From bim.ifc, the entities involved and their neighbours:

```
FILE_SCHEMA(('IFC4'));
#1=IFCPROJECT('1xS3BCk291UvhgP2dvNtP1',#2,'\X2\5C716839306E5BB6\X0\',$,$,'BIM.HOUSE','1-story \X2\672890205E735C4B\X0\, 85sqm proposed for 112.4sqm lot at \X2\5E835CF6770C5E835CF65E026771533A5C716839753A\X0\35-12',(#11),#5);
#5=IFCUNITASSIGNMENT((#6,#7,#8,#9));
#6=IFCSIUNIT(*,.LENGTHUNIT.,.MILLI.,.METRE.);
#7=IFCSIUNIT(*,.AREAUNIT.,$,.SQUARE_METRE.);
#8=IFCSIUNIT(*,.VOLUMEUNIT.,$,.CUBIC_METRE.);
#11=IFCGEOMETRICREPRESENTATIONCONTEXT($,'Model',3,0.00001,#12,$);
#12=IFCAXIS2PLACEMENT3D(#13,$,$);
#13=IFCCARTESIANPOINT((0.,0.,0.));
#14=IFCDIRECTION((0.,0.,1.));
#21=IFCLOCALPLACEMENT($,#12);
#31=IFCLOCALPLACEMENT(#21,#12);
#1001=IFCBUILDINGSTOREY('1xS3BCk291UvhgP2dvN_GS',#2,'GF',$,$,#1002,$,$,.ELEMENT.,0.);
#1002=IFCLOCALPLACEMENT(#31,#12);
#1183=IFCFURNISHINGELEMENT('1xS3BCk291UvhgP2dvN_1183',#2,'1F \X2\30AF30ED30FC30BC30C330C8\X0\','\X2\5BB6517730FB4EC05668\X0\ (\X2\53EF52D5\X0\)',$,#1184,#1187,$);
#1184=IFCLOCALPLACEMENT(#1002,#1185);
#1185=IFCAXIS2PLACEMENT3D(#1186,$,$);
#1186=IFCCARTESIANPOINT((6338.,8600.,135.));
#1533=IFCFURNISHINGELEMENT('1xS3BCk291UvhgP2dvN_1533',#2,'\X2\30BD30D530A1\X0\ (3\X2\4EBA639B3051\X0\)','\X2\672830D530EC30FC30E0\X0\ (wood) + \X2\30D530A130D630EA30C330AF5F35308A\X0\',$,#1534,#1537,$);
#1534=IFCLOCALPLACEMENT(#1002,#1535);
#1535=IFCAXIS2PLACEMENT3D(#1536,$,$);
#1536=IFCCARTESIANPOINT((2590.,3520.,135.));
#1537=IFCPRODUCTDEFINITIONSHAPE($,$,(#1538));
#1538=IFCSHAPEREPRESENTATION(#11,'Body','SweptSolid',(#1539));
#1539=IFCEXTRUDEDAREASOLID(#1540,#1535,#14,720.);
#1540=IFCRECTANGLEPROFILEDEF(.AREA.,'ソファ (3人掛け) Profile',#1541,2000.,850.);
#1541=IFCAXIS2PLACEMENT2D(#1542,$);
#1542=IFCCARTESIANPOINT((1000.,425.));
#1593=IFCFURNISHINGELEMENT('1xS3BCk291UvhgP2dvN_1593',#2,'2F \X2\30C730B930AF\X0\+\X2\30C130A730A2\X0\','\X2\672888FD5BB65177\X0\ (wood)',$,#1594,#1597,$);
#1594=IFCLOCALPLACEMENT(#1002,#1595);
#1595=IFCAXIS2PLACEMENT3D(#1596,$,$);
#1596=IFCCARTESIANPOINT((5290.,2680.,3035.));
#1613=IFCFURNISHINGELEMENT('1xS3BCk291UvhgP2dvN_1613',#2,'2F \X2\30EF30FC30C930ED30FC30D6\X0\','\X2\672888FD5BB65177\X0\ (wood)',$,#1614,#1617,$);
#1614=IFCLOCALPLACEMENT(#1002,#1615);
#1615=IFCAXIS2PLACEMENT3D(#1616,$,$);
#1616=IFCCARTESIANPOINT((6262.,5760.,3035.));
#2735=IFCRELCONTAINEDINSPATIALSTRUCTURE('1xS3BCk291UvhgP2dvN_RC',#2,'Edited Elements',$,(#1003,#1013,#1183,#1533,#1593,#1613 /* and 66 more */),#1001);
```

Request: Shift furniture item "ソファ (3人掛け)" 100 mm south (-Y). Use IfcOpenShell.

```python
import ifcopenshell
import ifcopenshell.api.geometry
import ifcopenshell.util.placement

model = ifcopenshell.open("bim.ifc")

item = model.by_id(1533)
matrix = ifcopenshell.util.placement.get_local_placement(item.ObjectPlacement)
matrix[1, 3] -= 100.0
ifcopenshell.api.geometry.edit_object_placement(model, product=item, matrix=matrix, is_si=False)

print(ifcopenshell.util.placement.get_local_placement(item.ObjectPlacement).round(3) + 0.0)

model.write("bim_updated.ifc")
```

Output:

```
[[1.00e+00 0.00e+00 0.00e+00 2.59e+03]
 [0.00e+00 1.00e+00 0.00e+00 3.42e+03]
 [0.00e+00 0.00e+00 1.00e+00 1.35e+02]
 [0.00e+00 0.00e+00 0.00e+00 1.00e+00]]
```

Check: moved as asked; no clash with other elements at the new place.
